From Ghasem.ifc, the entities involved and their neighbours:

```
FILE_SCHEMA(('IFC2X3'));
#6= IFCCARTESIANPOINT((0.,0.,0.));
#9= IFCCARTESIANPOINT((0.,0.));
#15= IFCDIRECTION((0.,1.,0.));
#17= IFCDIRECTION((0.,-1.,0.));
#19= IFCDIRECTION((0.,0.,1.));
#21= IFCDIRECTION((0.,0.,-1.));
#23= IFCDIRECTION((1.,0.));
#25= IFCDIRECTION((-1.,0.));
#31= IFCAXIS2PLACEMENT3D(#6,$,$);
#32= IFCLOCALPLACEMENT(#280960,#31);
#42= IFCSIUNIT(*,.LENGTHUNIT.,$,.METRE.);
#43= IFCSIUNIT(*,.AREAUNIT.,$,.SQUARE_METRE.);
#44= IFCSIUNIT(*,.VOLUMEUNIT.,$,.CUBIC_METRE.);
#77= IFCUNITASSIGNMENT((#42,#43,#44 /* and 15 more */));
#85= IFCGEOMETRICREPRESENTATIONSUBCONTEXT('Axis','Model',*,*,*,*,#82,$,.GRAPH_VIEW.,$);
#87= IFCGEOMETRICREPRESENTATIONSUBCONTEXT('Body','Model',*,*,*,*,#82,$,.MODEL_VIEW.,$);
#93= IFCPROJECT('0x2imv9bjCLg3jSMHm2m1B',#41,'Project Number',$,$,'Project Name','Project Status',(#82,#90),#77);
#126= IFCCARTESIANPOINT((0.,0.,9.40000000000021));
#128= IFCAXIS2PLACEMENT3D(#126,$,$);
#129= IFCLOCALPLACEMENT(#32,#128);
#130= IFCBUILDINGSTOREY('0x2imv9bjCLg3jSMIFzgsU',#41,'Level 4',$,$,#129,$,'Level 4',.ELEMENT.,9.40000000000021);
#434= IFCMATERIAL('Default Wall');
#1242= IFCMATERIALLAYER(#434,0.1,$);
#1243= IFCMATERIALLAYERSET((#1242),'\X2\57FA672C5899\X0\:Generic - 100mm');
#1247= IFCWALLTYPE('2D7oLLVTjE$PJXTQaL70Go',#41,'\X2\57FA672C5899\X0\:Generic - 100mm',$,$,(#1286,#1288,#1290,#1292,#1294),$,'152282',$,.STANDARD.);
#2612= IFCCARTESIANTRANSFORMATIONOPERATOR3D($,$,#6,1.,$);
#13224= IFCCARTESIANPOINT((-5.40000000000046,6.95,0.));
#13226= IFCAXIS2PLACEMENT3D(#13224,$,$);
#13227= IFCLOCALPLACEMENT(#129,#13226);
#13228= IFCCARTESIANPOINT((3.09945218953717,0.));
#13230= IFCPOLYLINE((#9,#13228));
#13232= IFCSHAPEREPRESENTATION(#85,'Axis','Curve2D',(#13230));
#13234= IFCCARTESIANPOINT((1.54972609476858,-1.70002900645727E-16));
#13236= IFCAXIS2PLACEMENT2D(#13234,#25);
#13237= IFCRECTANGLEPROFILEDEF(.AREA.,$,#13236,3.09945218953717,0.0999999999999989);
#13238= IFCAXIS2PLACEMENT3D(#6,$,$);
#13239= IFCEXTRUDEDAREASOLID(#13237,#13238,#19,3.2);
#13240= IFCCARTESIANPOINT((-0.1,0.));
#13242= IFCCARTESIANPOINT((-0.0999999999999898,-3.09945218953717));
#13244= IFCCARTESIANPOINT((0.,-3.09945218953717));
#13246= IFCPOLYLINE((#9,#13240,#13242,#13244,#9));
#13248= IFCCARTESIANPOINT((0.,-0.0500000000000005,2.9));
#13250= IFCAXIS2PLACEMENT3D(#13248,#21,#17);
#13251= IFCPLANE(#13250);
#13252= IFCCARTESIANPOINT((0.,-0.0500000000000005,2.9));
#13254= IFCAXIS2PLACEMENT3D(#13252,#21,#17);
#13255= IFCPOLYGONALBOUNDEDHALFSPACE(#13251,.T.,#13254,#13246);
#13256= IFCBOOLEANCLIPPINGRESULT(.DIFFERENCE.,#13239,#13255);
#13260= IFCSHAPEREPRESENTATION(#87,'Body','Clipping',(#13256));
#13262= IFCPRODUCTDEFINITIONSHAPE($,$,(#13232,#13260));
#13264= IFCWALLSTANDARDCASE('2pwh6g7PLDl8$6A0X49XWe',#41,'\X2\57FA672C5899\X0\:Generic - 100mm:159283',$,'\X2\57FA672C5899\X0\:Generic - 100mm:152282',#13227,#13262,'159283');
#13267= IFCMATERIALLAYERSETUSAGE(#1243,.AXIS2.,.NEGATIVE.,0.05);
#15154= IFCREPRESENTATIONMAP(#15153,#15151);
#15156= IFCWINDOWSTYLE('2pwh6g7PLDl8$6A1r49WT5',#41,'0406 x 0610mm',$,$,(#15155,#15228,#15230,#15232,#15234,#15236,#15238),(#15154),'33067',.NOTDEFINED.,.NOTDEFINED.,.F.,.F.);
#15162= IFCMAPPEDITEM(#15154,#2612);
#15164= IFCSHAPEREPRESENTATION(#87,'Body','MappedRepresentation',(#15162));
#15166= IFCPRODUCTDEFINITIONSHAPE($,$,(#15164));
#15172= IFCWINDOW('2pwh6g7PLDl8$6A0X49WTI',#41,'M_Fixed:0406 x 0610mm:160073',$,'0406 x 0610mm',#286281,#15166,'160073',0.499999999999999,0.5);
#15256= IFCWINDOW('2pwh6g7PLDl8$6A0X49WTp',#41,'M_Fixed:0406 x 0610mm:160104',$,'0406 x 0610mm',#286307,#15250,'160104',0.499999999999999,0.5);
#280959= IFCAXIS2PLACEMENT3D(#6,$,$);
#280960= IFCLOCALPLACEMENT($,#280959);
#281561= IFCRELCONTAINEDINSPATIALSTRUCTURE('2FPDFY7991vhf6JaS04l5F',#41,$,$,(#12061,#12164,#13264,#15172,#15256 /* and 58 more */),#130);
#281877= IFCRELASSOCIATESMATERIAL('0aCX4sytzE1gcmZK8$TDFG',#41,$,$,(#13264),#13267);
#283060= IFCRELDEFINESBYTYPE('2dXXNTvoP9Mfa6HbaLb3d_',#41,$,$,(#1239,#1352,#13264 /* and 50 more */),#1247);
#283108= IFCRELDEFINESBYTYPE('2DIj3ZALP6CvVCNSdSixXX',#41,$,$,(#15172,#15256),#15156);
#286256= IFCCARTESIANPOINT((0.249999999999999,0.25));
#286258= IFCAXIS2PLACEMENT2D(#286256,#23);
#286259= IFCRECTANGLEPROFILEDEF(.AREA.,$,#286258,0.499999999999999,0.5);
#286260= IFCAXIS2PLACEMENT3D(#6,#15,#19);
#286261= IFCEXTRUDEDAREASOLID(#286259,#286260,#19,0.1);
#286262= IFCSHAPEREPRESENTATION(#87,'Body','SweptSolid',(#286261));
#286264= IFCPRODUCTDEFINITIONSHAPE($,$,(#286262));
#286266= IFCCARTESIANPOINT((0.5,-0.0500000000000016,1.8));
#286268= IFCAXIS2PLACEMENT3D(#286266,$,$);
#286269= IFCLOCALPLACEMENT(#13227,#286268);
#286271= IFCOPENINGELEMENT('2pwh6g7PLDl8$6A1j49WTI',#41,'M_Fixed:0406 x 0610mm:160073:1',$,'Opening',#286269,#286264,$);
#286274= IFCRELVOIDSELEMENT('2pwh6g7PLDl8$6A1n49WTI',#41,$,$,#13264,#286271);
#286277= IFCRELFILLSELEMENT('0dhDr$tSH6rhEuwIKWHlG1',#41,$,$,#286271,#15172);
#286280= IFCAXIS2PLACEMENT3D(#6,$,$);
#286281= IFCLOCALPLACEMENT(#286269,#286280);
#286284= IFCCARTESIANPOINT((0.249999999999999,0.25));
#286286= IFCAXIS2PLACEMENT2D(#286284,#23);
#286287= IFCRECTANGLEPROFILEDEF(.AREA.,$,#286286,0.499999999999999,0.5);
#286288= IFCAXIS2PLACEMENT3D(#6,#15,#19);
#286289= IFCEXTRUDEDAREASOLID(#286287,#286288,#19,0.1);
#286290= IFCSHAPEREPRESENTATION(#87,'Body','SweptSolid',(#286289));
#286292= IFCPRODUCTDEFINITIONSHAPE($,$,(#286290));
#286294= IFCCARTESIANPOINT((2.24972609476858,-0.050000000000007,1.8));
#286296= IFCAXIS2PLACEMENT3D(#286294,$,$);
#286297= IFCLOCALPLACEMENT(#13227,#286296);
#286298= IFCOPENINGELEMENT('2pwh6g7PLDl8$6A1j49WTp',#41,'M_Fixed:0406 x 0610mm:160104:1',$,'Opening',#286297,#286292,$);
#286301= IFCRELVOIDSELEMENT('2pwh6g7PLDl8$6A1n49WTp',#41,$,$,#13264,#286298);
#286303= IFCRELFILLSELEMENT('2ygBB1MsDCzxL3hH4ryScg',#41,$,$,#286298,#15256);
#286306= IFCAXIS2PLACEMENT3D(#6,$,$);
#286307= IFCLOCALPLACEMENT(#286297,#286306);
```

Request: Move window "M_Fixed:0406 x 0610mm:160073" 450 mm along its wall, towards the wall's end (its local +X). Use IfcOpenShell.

```python
import ifcopenshell
import ifcopenshell.api.geometry
import ifcopenshell.util.placement

model = ifcopenshell.open("Ghasem.ifc")

window = model.by_guid("2pwh6g7PLDl8$6A0X49WTI")
opening = window.FillsVoids[0].RelatingOpeningElement
wall = opening.VoidsElements[0].RelatingBuildingElement

wall_matrix = ifcopenshell.util.placement.get_local_placement(wall.ObjectPlacement)
shift = wall_matrix[:3, 0] * 0.45
before = ifcopenshell.util.placement.get_local_placement(window.ObjectPlacement)[:3, 3].copy()

# The window is placed relative to its opening, so it follows when the opening moves.
matrix = ifcopenshell.util.placement.get_local_placement(opening.ObjectPlacement)
matrix[:3, 3] += shift
ifcopenshell.api.geometry.edit_object_placement(
    model, product=opening, matrix=matrix, is_si=False, should_transform_children=True
)

after = ifcopenshell.util.placement.get_local_placement(window.ObjectPlacement)[:3, 3]
print("window moved by", (after - before).round(3) + 0.0)

model.write("Ghasem_v2.ifc")
```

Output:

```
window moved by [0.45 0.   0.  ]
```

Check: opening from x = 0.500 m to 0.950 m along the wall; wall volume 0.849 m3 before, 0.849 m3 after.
